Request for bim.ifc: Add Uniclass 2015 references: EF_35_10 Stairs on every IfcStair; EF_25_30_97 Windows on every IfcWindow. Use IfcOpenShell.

First a look at what the model holds.

```python
import ifcopenshell

model = ifcopenshell.open("bim.ifc")
print(model.schema)
print("classifications:", [c.Name for c in model.by_type("IfcClassification")])
for ifc_class in ("IfcDoor", "IfcRoof", "IfcStair", "IfcWall", "IfcWindow"):
    print(ifc_class, len(model.by_type(ifc_class)))
```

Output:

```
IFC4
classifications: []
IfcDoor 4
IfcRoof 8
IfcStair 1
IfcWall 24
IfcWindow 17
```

```python
import ifcopenshell
import ifcopenshell.api.classification

model = ifcopenshell.open("bim.ifc")

system = ifcopenshell.api.classification.add_classification(model, classification="Uniclass 2015")

codes = {
    "IfcStair": ("EF_35_10", "Stairs"),
    "IfcWindow": ("EF_25_30_97", "Windows"),
}
for ifc_class, (code, name) in codes.items():
    products = model.by_type(ifc_class)
    ifcopenshell.api.classification.add_reference(
        model, products=products, classification=system, identification=code, name=name
    )
    print(code, len(products))

model.write("bim-out.ifc")
```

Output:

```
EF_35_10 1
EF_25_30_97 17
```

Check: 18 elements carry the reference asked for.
